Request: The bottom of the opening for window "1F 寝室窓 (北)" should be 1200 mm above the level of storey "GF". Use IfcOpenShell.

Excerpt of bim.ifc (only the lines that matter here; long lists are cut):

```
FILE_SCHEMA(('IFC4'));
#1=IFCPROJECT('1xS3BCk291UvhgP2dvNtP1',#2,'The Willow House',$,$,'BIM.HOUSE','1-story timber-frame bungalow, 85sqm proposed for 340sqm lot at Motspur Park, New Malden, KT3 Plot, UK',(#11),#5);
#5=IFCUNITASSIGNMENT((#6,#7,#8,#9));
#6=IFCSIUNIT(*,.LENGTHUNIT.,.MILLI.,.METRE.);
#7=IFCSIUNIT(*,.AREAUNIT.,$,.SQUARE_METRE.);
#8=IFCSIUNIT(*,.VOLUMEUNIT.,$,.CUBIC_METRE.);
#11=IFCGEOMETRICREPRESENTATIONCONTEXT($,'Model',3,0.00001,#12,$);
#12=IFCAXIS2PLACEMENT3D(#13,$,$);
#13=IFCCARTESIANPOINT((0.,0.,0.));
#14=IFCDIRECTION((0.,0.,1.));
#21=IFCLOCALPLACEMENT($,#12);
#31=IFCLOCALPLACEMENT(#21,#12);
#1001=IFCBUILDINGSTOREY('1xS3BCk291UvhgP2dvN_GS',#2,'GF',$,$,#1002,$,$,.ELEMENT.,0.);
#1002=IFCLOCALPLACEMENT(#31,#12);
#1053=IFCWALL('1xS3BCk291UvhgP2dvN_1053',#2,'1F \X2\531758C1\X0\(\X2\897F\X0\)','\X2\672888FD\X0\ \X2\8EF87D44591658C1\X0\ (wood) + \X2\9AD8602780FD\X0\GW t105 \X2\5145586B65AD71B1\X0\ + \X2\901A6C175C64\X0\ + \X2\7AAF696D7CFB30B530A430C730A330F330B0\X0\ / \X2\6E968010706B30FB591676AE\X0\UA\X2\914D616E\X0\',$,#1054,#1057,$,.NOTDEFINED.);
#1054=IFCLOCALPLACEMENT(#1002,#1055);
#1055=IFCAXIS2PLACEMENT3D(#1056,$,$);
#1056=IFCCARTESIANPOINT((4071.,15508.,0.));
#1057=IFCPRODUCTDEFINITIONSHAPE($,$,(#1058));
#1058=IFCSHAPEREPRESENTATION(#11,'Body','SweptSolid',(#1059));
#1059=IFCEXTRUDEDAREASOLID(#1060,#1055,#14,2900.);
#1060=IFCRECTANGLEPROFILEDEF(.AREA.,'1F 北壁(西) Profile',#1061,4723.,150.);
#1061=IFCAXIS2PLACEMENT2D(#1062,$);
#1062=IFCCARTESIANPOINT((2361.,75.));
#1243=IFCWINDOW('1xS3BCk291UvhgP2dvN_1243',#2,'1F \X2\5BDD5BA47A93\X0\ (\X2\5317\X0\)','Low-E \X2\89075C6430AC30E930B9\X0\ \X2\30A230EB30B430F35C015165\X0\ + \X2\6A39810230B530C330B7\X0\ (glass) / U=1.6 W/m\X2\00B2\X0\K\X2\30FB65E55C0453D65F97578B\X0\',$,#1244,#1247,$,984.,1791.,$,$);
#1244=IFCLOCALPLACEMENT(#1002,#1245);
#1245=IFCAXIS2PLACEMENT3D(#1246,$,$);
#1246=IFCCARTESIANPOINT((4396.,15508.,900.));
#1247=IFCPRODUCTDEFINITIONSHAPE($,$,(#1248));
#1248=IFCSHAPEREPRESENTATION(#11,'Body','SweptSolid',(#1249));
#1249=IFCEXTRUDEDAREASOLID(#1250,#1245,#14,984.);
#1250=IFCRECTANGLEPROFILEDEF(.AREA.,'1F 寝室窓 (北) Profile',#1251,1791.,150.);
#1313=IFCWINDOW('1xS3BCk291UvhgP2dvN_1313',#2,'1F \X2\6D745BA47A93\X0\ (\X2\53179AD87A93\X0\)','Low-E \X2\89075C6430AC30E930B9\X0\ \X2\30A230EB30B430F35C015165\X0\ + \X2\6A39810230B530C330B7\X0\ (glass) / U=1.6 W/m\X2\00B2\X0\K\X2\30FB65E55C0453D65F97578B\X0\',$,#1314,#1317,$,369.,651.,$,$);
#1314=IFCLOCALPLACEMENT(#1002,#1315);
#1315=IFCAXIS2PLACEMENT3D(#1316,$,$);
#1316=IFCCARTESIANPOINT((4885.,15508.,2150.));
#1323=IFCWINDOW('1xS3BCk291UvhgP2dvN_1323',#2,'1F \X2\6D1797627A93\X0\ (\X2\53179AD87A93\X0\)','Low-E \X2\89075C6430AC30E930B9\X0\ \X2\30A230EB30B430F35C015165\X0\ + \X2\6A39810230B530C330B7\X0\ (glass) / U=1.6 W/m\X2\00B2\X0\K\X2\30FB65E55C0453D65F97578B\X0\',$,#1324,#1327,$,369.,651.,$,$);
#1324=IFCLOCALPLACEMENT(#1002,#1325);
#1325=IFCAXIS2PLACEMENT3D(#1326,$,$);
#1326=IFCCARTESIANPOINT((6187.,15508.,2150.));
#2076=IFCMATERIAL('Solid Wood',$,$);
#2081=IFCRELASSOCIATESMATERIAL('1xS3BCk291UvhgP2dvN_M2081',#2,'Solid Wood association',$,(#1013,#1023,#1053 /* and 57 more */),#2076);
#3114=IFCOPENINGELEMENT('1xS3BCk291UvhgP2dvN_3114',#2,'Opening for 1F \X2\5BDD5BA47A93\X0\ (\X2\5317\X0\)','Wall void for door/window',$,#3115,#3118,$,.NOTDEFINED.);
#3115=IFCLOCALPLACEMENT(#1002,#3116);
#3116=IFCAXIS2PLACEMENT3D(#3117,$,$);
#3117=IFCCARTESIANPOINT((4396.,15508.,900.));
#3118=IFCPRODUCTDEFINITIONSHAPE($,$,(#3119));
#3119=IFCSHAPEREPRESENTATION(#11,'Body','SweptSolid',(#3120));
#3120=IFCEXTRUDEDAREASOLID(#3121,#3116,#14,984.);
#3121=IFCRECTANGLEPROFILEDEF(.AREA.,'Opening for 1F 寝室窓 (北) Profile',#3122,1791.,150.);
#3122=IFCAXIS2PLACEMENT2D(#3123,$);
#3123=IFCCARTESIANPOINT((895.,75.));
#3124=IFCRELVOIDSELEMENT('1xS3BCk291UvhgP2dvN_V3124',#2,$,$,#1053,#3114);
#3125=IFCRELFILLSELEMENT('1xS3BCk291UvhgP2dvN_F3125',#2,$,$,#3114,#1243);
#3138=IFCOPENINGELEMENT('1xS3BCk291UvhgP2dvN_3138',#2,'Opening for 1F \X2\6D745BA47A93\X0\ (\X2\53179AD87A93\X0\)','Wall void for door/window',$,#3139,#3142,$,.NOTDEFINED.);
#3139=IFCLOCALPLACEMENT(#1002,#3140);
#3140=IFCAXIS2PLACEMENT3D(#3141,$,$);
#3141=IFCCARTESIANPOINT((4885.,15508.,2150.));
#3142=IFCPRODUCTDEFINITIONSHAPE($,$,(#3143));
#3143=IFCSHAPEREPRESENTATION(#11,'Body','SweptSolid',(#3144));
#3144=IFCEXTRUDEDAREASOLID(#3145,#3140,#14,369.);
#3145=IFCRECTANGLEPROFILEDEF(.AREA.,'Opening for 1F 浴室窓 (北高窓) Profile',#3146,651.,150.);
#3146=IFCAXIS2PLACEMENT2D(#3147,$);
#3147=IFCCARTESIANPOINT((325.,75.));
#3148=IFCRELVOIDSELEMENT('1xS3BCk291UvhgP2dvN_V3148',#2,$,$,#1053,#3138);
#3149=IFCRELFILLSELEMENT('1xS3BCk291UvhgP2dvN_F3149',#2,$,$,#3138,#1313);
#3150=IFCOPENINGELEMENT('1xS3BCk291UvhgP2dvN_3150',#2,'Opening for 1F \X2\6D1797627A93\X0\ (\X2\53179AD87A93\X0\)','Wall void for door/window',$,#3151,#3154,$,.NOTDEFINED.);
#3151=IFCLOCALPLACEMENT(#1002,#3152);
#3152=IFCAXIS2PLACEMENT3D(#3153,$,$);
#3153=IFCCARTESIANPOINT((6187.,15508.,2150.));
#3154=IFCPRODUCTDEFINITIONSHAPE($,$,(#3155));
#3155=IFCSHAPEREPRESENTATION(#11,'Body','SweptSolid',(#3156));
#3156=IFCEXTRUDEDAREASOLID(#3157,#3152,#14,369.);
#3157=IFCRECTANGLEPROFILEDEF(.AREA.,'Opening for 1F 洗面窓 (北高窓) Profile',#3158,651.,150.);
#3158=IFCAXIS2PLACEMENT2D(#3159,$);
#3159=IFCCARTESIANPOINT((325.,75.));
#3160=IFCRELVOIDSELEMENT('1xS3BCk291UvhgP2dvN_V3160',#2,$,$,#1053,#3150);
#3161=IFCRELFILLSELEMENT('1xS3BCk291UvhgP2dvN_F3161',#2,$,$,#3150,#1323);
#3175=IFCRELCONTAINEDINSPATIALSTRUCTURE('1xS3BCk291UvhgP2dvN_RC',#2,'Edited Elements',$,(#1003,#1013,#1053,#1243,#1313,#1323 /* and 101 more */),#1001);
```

```python
import numpy as np
import ifcopenshell
import ifcopenshell.api.geometry
import ifcopenshell.geom
import ifcopenshell.util.element
import ifcopenshell.util.placement
import ifcopenshell.util.shape
import ifcopenshell.util.unit

model = ifcopenshell.open("bim.ifc")
unit_scale = ifcopenshell.util.unit.calculate_unit_scale(model)

window = model.by_guid("1xS3BCk291UvhgP2dvN_1243")
opening = window.FillsVoids[0].RelatingOpeningElement
storey = ifcopenshell.util.element.get_container(window, ifc_class="IfcBuildingStorey")
level = ifcopenshell.util.placement.get_local_placement(storey.ObjectPlacement)[2, 3]

# The opening's origin need not be at the sill, so measure its lowest point.
shape = ifcopenshell.geom.create_shape(ifcopenshell.geom.settings(), opening)
bottom = ifcopenshell.util.shape.get_shape_bottom_elevation(shape, shape.geometry) / unit_scale
dz = level + 1.2 / unit_scale - bottom

shift = np.array([0.0, 0.0, dz])
# The window is not placed relative to its opening, so move both.
for product in (opening, window):
    matrix = ifcopenshell.util.placement.get_local_placement(product.ObjectPlacement)
    matrix[:3, 3] += shift
    ifcopenshell.api.geometry.edit_object_placement(model, product=product, matrix=matrix, is_si=False)

print(f"moved by {dz * unit_scale:+.3f} m")

model.write("bim_rev.ifc")
```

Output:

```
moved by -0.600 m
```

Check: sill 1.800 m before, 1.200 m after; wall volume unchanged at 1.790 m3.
